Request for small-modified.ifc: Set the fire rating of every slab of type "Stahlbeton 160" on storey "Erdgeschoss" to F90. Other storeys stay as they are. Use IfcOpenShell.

First a look at what the model holds.

```python
import ifcopenshell
import ifcopenshell.util.element

model = ifcopenshell.open("small-modified.ifc")
print(model.schema)
storey = next(s for s in model.by_type("IfcBuildingStorey") if s.Name == "Erdgeschoss")
slabs = [e for e in ifcopenshell.util.element.get_decomposition(storey) if e.is_a("IfcSlab")]
seen = {}
for e in slabs:
    element_type = ifcopenshell.util.element.get_type(e)
    key = (element_type.Name if element_type != e and element_type else None, ifcopenshell.util.element.get_pset(e, "Pset_SlabCommon", "FireRating"))
    seen[key] = seen.get(key, 0) + 1
for (name, value), count in sorted(seen.items(), key=str):
    print(count, "x", name, "|", value)
```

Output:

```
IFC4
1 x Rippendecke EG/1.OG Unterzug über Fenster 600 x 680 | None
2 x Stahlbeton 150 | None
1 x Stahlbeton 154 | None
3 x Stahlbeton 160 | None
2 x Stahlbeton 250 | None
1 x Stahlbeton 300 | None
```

```python
import ifcopenshell
import ifcopenshell.api.pset
import ifcopenshell.util.element

model = ifcopenshell.open("small-modified.ifc")

storey = next(s for s in model.by_type("IfcBuildingStorey") if s.Name == "Erdgeschoss")
slabs = [e for e in ifcopenshell.util.element.get_decomposition(storey) if e.is_a("IfcSlab")]

count = 0
for e in slabs:
    element_type = ifcopenshell.util.element.get_type(e)
    if element_type in (None, e) or element_type.Name != "Stahlbeton 160":
        continue
    # add_pset returns the element's existing set when there is one.
    pset = ifcopenshell.api.pset.add_pset(model, product=e, name="Pset_SlabCommon")
    ifcopenshell.api.pset.edit_pset(model, pset=pset, properties={"FireRating": "F90"})
    count += 1

print(count, "slabs updated")

model.write("small-modified_v2.ifc")
```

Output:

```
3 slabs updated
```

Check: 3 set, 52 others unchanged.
